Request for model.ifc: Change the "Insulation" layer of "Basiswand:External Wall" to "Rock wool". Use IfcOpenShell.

First a look at what the model holds.

```python
import ifcopenshell
import ifcopenshell.util.element

model = ifcopenshell.open("model.ifc")
print(model.schema)
for layer_set in model.by_type("IfcMaterialLayerSet"):
    if layer_set.LayerSetName == "Basiswand:External Wall":
        for layer in layer_set.MaterialLayers:
            print(layer.id(), layer.Material and layer.Material.Name, layer.LayerThickness, sep=" | ")
        print(len(ifcopenshell.util.element.get_elements_by_material(model, layer_set)), "elements and types use it")
print(sorted(m.Name for m in model.by_type("IfcMaterial") if m.Name)[:60])
```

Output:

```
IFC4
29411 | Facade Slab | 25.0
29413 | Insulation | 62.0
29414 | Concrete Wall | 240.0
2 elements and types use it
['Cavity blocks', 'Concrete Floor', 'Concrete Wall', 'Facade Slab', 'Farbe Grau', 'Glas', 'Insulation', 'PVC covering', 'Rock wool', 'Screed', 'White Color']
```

```python
import ifcopenshell
import ifcopenshell.api.material

model = ifcopenshell.open("model.ifc")

layer_set = next(s for s in model.by_type("IfcMaterialLayerSet") if s.LayerSetName == "Basiswand:External Wall")
layer = next(l for l in layer_set.MaterialLayers if l.Material and l.Material.Name == "Insulation")
material = next(m for m in model.by_type("IfcMaterial") if m.Name == "Rock wool")

# Point this one layer at the other material; renaming the old one would change it everywhere.
ifcopenshell.api.material.edit_layer(model, layer=layer, attributes={}, material=material)

print([l.Material.Name if l.Material else None for l in layer_set.MaterialLayers])

model.write("model_updated.ifc")
```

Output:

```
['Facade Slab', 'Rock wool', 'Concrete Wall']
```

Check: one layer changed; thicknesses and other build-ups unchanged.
